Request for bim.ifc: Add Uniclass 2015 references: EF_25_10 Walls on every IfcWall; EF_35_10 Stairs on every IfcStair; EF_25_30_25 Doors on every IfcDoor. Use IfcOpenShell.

First a look at what the model holds.

```python
import ifcopenshell

model = ifcopenshell.open("bim.ifc")
print(model.schema)
print("classifications:", [c.Name for c in model.by_type("IfcClassification")])
for ifc_class in ("IfcDoor", "IfcRoof", "IfcStair", "IfcWall", "IfcWindow"):
    print(ifc_class, len(model.by_type(ifc_class)))
```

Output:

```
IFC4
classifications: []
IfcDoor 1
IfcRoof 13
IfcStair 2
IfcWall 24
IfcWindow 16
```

```python
import ifcopenshell
import ifcopenshell.api.classification

model = ifcopenshell.open("bim.ifc")

system = ifcopenshell.api.classification.add_classification(model, classification="Uniclass 2015")

codes = {
    "IfcWall": ("EF_25_10", "Walls"),
    "IfcStair": ("EF_35_10", "Stairs"),
    "IfcDoor": ("EF_25_30_25", "Doors"),
}
for ifc_class, (code, name) in codes.items():
    products = model.by_type(ifc_class)
    ifcopenshell.api.classification.add_reference(
        model, products=products, classification=system, identification=code, name=name
    )
    print(code, len(products))

model.write("bim_updated.ifc")
```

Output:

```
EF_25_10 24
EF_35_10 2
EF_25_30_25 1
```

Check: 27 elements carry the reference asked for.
